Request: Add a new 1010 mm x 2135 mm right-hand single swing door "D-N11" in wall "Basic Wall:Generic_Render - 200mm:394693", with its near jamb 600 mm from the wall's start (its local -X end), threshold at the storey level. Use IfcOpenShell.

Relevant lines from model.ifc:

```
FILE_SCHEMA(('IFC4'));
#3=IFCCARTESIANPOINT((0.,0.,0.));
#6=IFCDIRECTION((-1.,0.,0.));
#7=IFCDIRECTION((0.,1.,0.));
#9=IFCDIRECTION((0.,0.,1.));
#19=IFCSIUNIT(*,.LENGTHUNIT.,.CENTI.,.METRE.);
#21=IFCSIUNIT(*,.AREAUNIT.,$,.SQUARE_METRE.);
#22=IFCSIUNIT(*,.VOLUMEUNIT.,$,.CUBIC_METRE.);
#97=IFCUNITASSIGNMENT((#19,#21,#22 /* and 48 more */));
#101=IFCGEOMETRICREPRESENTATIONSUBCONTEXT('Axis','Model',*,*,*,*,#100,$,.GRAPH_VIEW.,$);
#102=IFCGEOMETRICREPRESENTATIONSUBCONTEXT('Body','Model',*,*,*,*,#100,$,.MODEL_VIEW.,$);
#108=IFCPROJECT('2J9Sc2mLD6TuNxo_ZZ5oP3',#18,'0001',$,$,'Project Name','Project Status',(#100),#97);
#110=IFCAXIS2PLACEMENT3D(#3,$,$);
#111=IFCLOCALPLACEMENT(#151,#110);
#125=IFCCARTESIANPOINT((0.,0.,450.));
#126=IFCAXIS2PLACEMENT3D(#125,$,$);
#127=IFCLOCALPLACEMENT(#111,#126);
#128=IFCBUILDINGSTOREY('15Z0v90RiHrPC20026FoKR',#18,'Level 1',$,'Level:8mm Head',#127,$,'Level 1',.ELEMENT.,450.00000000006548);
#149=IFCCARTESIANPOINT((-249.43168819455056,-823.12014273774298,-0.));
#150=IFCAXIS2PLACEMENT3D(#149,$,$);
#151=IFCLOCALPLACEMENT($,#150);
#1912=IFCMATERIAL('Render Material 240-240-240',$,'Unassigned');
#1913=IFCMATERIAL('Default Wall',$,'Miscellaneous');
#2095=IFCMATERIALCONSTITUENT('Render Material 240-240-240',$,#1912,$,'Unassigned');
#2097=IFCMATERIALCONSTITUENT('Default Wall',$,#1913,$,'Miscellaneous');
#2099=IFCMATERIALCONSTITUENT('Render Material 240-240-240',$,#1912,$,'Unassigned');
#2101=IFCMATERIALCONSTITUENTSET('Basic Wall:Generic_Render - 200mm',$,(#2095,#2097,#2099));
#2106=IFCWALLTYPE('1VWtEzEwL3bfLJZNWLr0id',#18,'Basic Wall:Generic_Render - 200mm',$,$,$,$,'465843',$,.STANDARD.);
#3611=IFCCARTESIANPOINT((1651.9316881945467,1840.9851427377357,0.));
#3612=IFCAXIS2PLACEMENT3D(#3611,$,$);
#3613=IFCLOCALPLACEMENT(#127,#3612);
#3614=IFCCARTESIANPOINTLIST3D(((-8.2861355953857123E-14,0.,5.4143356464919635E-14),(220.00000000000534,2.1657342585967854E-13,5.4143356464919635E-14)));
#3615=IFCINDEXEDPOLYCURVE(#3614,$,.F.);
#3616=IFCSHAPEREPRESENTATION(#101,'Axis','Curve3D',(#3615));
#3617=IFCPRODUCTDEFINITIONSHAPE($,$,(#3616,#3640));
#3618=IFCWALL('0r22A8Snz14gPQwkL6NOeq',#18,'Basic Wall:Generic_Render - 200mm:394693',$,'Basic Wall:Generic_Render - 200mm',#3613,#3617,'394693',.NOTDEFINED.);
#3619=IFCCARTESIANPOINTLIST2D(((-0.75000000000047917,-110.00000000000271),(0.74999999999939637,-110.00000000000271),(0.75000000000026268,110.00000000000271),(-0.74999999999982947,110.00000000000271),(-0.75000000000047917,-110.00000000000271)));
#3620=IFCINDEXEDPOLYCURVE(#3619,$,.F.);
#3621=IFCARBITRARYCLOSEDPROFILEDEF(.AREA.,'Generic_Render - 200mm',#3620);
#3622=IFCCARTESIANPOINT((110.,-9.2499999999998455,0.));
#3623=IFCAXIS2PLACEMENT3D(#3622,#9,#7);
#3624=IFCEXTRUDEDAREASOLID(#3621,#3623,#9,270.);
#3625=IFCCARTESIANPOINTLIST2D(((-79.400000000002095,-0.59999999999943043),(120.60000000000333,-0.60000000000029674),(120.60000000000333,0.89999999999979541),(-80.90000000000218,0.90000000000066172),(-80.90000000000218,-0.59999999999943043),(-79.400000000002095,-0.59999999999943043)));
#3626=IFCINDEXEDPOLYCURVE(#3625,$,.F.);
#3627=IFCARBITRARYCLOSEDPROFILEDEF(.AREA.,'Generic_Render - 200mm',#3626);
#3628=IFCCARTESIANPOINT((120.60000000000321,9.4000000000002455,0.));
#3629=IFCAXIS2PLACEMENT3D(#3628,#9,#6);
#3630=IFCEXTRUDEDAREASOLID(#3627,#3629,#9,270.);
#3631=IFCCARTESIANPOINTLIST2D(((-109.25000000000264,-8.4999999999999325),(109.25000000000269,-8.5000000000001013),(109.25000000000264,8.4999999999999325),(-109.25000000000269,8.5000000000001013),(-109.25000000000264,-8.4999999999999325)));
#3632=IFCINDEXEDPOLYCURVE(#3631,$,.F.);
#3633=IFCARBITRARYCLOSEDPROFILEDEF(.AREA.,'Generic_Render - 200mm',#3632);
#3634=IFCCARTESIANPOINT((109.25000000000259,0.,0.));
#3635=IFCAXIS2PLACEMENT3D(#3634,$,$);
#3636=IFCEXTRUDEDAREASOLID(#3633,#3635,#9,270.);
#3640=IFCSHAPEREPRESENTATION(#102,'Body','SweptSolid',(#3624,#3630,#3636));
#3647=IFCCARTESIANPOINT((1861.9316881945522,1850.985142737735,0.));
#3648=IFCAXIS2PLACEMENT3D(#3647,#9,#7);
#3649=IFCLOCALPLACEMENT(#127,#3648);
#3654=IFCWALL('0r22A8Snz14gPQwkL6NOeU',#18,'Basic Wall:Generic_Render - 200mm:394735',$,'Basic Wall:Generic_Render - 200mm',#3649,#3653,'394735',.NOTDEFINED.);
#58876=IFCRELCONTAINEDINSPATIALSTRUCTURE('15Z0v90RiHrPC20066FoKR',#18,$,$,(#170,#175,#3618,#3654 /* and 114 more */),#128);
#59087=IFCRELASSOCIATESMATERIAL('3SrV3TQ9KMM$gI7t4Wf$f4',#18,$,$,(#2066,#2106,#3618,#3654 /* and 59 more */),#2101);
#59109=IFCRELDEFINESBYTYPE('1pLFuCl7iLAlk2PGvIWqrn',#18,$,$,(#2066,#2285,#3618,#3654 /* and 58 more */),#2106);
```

```python
import numpy as np
import ifcopenshell
import ifcopenshell.api.feature
import ifcopenshell.api.geometry
import ifcopenshell.api.root
import ifcopenshell.api.spatial
import ifcopenshell.geom
import ifcopenshell.util.element
import ifcopenshell.util.placement
import ifcopenshell.util.representation
import ifcopenshell.util.shape
import ifcopenshell.util.unit

model = ifcopenshell.open("model.ifc")
unit_scale = ifcopenshell.util.unit.calculate_unit_scale(model)
settings = ifcopenshell.geom.settings()


def volume(element):
    """Net volume in cubic metres, openings subtracted."""
    shape = ifcopenshell.geom.create_shape(settings, element)
    return ifcopenshell.util.shape.get_volume(shape.geometry)


wall = model.by_guid("0r22A8Snz14gPQwkL6NOeq")
storey = ifcopenshell.util.element.get_container(wall, ifc_class="IfcBuildingStorey")
context = ifcopenshell.util.representation.get_context(model, "Model", "Body", "MODEL_VIEW")
before = volume(wall)

width, height, from_end, sill = 1.01, 2.135, 0.6, 0.0  # metres

# The wall runs along its own X axis, and the end named is its -X end.
wall_shape = ifcopenshell.geom.create_shape(settings, wall)
x, y, z = ifcopenshell.util.shape.get_vertices(wall_shape.geometry).T
start = x.min() + from_end
face, thickness = float(y.min()), float(y.max() - y.min())
wall_matrix = ifcopenshell.util.placement.get_local_placement(wall.ObjectPlacement)
level = ifcopenshell.util.placement.get_local_placement(storey.ObjectPlacement)[2, 3]


def in_wall(x, y):
    """Placement at x, y metres in the wall's axes, at sill height."""
    matrix = wall_matrix.copy()
    matrix[:, 3] = wall_matrix @ np.array([x / unit_scale, y / unit_scale, 0.0, 1.0])
    matrix[2, 3] = level + sill / unit_scale
    return matrix


# Opening: a box that overshoots both wall faces by 50 mm.
opening = ifcopenshell.api.root.create_entity(model, ifc_class="IfcOpeningElement", predefined_type="OPENING")
box = ifcopenshell.api.geometry.add_wall_representation(
    model, context=context, length=width, height=height, thickness=thickness + 0.1
)
ifcopenshell.api.geometry.assign_representation(model, product=opening, representation=box)
ifcopenshell.api.geometry.edit_object_placement(model, product=opening, matrix=in_wall(start, face - 0.05), is_si=False)
ifcopenshell.api.feature.add_feature(model, feature=opening, element=wall)

door = ifcopenshell.api.root.create_entity(model, ifc_class="IfcDoor", name="D-N11", predefined_type="DOOR")
door.OverallWidth, door.OverallHeight = width / unit_scale, height / unit_scale
door.OperationType = "SINGLE_SWING_RIGHT"
body = ifcopenshell.api.geometry.add_door_representation(
    model,
    context=context,
    overall_width=door.OverallWidth,
    overall_height=door.OverallHeight,
    operation_type="SINGLE_SWING_RIGHT",
    lining_properties={"LiningDepth": thickness / unit_scale, "ThresholdDepth": thickness / unit_scale},
)
ifcopenshell.api.geometry.assign_representation(model, product=door, representation=body)
ifcopenshell.api.spatial.assign_container(model, products=[door], relating_structure=storey)
ifcopenshell.api.feature.add_filling(model, opening=opening, element=door)

# The lining spans the wall, so the door starts at the wall face.
ifcopenshell.api.geometry.edit_object_placement(model, product=door, matrix=in_wall(start, face), is_si=False)

after = volume(wall)

print(f"wall volume {before:.3f} -> {after:.3f} m3")

model.write("model_updated.ifc")
```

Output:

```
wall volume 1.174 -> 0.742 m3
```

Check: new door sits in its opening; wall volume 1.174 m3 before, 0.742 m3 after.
